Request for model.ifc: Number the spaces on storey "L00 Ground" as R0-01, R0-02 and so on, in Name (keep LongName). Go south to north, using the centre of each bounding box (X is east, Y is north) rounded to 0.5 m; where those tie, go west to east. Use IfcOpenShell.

First a look at what the model holds.

```python
import ifcopenshell
import ifcopenshell.util.element
import ifcopenshell.util.placement

model = ifcopenshell.open("model.ifc")
print(model.schema)
storey = next(s for s in model.by_type("IfcBuildingStorey") if s.Name == "L00 Ground")
spaces = [e for e in ifcopenshell.util.element.get_decomposition(storey) if e.is_a("IfcSpace")]
for e in sorted(spaces, key=lambda e: e.id()):
    origin = ifcopenshell.util.placement.get_local_placement(e.ObjectPlacement)[:3, 3]
    print(e.id(), e.Name, e.LongName, origin.round(2) + 0.0, sep=" | ")
```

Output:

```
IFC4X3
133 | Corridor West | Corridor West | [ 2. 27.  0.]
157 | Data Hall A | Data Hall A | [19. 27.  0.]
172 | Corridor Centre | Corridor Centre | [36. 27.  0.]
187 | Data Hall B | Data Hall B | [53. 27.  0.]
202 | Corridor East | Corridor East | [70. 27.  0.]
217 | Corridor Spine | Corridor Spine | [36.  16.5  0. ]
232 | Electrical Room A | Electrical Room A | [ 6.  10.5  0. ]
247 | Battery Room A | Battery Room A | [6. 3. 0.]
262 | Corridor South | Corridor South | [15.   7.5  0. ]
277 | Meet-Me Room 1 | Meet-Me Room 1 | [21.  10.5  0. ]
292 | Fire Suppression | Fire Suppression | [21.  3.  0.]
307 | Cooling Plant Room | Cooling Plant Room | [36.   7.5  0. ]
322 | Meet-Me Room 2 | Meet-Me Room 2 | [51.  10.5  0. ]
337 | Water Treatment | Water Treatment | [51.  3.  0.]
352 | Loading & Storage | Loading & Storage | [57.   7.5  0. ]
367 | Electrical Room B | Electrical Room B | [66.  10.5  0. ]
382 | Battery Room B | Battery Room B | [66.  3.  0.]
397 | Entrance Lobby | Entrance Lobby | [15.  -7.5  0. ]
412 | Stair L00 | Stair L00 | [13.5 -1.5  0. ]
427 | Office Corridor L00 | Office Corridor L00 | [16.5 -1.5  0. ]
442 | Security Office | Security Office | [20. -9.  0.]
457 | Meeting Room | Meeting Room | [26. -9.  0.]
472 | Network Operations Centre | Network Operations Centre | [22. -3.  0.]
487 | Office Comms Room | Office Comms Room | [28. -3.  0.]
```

```python
import ifcopenshell
import ifcopenshell.geom
import ifcopenshell.util.element
import ifcopenshell.util.shape

model = ifcopenshell.open("model.ifc")
settings = ifcopenshell.geom.settings()
settings.set("use-world-coords", True)


def centre(element):
    shape = ifcopenshell.geom.create_shape(settings, element)
    return ifcopenshell.util.shape.get_bbox_centroid(shape.geometry)


storey = next(s for s in model.by_type("IfcBuildingStorey") if s.Name == "L00 Ground")
spaces = [e for e in ifcopenshell.util.element.get_decomposition(storey) if e.is_a("IfcSpace")]

# Insertion points can sit at a corner or the storey origin, so sort by the geometry (in metres).
centres = {e: centre(e) for e in spaces}
spaces.sort(key=lambda e: (round(centres[e][1] / 0.5), centres[e][0]))

for i, e in enumerate(spaces, start=1):
    number = f"R0-{i:02d}"
    e.Name = number
    print(e.id(), number)

model.write("model_updated.ifc")
```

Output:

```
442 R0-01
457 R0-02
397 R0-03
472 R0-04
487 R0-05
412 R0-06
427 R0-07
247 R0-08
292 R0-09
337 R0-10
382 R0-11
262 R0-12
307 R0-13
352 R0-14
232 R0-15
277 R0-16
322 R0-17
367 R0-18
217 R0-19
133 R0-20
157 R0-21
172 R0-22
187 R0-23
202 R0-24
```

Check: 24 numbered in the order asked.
